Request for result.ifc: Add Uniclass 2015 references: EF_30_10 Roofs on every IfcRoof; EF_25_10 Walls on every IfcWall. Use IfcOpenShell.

First a look at what the model holds.

```python
import ifcopenshell

model = ifcopenshell.open("result.ifc")
print(model.schema)
print("classifications:", [c.Name for c in model.by_type("IfcClassification")])
for ifc_class in ("IfcDoor", "IfcRoof", "IfcStair", "IfcWall", "IfcWindow"):
    print(ifc_class, len(model.by_type(ifc_class)))
```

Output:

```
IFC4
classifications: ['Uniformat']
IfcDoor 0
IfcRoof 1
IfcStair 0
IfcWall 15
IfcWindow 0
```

```python
import ifcopenshell
import ifcopenshell.api.classification

model = ifcopenshell.open("result.ifc")

system = ifcopenshell.api.classification.add_classification(model, classification="Uniclass 2015")

codes = {
    "IfcRoof": ("EF_30_10", "Roofs"),
    "IfcWall": ("EF_25_10", "Walls"),
}
for ifc_class, (code, name) in codes.items():
    products = model.by_type(ifc_class)
    ifcopenshell.api.classification.add_reference(
        model, products=products, classification=system, identification=code, name=name
    )
    print(code, len(products))

model.write("result_updated.ifc")
```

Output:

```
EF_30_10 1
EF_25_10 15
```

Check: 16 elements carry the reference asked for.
